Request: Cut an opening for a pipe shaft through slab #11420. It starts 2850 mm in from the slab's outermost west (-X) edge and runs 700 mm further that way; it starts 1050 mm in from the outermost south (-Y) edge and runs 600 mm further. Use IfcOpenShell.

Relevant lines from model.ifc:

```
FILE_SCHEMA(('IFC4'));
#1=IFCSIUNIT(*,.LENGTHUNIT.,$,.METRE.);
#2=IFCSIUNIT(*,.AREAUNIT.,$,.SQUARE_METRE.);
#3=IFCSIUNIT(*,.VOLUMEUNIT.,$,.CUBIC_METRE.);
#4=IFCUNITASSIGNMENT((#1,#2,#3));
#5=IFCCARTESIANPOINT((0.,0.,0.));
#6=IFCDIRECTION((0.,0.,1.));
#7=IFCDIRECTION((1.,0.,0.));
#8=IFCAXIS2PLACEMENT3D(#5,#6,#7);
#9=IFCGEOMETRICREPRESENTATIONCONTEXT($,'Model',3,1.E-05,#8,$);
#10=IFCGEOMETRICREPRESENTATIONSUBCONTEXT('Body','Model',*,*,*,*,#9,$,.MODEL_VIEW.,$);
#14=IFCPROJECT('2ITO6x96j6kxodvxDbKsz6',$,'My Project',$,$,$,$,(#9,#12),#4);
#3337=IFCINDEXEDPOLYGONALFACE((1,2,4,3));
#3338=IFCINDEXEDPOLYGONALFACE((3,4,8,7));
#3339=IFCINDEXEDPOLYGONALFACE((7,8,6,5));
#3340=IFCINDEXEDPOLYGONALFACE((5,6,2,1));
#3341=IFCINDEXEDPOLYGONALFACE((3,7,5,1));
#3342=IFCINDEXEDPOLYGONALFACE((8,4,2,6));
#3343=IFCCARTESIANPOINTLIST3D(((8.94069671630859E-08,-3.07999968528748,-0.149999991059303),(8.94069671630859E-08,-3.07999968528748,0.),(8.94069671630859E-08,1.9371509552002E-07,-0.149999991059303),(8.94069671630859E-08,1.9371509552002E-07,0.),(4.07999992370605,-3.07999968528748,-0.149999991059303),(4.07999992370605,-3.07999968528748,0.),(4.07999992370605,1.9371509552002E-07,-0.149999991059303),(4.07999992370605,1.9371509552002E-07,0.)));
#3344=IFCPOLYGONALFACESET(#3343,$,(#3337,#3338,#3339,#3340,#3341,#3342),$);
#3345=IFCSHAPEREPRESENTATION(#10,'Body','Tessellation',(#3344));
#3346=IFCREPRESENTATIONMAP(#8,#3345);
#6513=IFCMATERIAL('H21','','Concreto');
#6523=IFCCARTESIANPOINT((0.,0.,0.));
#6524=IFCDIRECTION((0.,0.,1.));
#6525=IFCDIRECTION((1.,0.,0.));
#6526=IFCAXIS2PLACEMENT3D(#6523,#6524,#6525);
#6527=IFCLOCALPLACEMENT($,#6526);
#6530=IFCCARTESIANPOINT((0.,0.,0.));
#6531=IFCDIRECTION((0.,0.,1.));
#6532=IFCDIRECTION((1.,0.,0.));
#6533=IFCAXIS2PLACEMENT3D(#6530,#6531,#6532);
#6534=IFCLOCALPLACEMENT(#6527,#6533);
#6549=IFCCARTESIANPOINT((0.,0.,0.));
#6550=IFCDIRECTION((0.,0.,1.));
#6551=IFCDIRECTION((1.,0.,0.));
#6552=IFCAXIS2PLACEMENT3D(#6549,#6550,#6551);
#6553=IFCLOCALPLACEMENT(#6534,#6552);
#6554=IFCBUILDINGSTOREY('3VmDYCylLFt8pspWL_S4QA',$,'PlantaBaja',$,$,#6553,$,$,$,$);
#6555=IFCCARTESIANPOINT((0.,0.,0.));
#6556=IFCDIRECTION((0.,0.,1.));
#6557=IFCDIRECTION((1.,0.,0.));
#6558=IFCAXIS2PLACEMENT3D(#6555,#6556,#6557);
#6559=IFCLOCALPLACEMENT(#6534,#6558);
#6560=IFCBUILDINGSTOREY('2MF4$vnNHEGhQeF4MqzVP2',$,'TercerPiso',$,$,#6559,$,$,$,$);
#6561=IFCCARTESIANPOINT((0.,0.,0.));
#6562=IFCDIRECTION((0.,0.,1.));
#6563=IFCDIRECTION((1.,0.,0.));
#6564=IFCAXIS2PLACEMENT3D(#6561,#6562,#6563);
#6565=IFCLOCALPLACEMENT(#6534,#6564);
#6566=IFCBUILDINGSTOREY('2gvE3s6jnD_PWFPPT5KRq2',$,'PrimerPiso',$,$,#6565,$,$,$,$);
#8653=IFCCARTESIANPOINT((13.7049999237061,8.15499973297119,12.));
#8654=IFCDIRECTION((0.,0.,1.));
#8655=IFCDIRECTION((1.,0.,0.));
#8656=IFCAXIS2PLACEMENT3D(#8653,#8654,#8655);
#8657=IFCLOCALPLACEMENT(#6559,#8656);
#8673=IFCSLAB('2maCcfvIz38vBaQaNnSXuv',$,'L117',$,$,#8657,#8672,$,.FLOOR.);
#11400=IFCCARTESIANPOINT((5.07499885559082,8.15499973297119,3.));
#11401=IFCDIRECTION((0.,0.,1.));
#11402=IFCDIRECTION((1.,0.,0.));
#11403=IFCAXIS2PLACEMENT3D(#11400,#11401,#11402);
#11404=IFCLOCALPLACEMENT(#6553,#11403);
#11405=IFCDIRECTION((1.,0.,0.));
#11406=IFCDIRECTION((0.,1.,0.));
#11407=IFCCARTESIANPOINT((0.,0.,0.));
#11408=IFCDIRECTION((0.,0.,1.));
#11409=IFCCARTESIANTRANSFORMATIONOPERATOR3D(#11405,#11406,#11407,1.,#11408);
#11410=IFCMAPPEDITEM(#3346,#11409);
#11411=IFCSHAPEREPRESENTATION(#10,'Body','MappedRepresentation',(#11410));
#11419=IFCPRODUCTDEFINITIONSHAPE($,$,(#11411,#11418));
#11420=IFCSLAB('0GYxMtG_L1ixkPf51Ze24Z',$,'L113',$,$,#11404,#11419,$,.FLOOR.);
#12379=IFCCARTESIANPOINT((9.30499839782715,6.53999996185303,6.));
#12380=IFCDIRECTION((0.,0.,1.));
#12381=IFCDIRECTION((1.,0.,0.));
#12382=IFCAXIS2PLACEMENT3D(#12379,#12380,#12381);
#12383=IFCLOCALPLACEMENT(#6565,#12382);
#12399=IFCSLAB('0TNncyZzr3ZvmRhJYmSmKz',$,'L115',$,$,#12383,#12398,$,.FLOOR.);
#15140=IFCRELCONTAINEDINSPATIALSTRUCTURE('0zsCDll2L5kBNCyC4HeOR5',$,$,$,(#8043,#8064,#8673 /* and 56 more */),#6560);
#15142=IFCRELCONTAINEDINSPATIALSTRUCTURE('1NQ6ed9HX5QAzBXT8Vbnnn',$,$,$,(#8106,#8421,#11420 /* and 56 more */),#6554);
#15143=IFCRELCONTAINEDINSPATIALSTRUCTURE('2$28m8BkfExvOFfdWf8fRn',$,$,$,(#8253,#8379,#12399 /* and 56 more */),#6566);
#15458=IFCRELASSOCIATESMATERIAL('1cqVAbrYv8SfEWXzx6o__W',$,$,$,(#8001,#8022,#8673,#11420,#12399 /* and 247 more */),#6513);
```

```python
import numpy as np
import ifcopenshell
import ifcopenshell.api.feature
import ifcopenshell.api.geometry
import ifcopenshell.api.root
import ifcopenshell.geom
import ifcopenshell.util.placement
import ifcopenshell.util.representation
import ifcopenshell.util.shape
import ifcopenshell.util.unit

model = ifcopenshell.open("model.ifc")
unit_scale = ifcopenshell.util.unit.calculate_unit_scale(model)
settings = ifcopenshell.geom.settings()


def volume(element):
    """Net volume in cubic metres, openings subtracted."""
    shape = ifcopenshell.geom.create_shape(settings, element)
    return ifcopenshell.util.shape.get_volume(shape.geometry)


slab = model.by_guid("0GYxMtG_L1ixkPf51Ze24Z")
before = volume(slab)

# Extent in the slab's own axes, in metres. The edges named are its -X and -Y sides.
slab_shape = ifcopenshell.geom.create_shape(settings, slab)
vertices = ifcopenshell.util.shape.get_vertices(slab_shape.geometry)
x_min, y_min, bottom = vertices.min(axis=0)
top = vertices[:, 2].max()

opening = ifcopenshell.api.root.create_entity(model, ifc_class="IfcOpeningElement", name="Pipe shaft opening", predefined_type="OPENING")
context = ifcopenshell.util.representation.get_context(model, "Model", "Body", "MODEL_VIEW")
width, depth = 0.7, 0.6
outline = [(0.0, 0.0), (width, 0.0), (width, depth), (0.0, depth), (0.0, 0.0)]
# Overshoot both faces by 50 mm so the cut is clean.
shape = ifcopenshell.api.geometry.add_slab_representation(
    model, context=context, depth=top - bottom + 0.1, polyline=outline
)
ifcopenshell.api.geometry.assign_representation(model, product=opening, representation=shape)

matrix = ifcopenshell.util.placement.get_local_placement(slab.ObjectPlacement)
matrix[:, 3] = matrix @ np.append(np.array([x_min + 2.85, y_min + 1.05, bottom - 0.05]) / unit_scale, 1.0)
ifcopenshell.api.geometry.edit_object_placement(model, product=opening, matrix=matrix, is_si=False)
ifcopenshell.api.feature.add_feature(model, feature=opening, element=slab)

after = volume(slab)

print(f"slab volume {before:.3f} -> {after:.3f} m3")

model.write("model_edited.ifc")
```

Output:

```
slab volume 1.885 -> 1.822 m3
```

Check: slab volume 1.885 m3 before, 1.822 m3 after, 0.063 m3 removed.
